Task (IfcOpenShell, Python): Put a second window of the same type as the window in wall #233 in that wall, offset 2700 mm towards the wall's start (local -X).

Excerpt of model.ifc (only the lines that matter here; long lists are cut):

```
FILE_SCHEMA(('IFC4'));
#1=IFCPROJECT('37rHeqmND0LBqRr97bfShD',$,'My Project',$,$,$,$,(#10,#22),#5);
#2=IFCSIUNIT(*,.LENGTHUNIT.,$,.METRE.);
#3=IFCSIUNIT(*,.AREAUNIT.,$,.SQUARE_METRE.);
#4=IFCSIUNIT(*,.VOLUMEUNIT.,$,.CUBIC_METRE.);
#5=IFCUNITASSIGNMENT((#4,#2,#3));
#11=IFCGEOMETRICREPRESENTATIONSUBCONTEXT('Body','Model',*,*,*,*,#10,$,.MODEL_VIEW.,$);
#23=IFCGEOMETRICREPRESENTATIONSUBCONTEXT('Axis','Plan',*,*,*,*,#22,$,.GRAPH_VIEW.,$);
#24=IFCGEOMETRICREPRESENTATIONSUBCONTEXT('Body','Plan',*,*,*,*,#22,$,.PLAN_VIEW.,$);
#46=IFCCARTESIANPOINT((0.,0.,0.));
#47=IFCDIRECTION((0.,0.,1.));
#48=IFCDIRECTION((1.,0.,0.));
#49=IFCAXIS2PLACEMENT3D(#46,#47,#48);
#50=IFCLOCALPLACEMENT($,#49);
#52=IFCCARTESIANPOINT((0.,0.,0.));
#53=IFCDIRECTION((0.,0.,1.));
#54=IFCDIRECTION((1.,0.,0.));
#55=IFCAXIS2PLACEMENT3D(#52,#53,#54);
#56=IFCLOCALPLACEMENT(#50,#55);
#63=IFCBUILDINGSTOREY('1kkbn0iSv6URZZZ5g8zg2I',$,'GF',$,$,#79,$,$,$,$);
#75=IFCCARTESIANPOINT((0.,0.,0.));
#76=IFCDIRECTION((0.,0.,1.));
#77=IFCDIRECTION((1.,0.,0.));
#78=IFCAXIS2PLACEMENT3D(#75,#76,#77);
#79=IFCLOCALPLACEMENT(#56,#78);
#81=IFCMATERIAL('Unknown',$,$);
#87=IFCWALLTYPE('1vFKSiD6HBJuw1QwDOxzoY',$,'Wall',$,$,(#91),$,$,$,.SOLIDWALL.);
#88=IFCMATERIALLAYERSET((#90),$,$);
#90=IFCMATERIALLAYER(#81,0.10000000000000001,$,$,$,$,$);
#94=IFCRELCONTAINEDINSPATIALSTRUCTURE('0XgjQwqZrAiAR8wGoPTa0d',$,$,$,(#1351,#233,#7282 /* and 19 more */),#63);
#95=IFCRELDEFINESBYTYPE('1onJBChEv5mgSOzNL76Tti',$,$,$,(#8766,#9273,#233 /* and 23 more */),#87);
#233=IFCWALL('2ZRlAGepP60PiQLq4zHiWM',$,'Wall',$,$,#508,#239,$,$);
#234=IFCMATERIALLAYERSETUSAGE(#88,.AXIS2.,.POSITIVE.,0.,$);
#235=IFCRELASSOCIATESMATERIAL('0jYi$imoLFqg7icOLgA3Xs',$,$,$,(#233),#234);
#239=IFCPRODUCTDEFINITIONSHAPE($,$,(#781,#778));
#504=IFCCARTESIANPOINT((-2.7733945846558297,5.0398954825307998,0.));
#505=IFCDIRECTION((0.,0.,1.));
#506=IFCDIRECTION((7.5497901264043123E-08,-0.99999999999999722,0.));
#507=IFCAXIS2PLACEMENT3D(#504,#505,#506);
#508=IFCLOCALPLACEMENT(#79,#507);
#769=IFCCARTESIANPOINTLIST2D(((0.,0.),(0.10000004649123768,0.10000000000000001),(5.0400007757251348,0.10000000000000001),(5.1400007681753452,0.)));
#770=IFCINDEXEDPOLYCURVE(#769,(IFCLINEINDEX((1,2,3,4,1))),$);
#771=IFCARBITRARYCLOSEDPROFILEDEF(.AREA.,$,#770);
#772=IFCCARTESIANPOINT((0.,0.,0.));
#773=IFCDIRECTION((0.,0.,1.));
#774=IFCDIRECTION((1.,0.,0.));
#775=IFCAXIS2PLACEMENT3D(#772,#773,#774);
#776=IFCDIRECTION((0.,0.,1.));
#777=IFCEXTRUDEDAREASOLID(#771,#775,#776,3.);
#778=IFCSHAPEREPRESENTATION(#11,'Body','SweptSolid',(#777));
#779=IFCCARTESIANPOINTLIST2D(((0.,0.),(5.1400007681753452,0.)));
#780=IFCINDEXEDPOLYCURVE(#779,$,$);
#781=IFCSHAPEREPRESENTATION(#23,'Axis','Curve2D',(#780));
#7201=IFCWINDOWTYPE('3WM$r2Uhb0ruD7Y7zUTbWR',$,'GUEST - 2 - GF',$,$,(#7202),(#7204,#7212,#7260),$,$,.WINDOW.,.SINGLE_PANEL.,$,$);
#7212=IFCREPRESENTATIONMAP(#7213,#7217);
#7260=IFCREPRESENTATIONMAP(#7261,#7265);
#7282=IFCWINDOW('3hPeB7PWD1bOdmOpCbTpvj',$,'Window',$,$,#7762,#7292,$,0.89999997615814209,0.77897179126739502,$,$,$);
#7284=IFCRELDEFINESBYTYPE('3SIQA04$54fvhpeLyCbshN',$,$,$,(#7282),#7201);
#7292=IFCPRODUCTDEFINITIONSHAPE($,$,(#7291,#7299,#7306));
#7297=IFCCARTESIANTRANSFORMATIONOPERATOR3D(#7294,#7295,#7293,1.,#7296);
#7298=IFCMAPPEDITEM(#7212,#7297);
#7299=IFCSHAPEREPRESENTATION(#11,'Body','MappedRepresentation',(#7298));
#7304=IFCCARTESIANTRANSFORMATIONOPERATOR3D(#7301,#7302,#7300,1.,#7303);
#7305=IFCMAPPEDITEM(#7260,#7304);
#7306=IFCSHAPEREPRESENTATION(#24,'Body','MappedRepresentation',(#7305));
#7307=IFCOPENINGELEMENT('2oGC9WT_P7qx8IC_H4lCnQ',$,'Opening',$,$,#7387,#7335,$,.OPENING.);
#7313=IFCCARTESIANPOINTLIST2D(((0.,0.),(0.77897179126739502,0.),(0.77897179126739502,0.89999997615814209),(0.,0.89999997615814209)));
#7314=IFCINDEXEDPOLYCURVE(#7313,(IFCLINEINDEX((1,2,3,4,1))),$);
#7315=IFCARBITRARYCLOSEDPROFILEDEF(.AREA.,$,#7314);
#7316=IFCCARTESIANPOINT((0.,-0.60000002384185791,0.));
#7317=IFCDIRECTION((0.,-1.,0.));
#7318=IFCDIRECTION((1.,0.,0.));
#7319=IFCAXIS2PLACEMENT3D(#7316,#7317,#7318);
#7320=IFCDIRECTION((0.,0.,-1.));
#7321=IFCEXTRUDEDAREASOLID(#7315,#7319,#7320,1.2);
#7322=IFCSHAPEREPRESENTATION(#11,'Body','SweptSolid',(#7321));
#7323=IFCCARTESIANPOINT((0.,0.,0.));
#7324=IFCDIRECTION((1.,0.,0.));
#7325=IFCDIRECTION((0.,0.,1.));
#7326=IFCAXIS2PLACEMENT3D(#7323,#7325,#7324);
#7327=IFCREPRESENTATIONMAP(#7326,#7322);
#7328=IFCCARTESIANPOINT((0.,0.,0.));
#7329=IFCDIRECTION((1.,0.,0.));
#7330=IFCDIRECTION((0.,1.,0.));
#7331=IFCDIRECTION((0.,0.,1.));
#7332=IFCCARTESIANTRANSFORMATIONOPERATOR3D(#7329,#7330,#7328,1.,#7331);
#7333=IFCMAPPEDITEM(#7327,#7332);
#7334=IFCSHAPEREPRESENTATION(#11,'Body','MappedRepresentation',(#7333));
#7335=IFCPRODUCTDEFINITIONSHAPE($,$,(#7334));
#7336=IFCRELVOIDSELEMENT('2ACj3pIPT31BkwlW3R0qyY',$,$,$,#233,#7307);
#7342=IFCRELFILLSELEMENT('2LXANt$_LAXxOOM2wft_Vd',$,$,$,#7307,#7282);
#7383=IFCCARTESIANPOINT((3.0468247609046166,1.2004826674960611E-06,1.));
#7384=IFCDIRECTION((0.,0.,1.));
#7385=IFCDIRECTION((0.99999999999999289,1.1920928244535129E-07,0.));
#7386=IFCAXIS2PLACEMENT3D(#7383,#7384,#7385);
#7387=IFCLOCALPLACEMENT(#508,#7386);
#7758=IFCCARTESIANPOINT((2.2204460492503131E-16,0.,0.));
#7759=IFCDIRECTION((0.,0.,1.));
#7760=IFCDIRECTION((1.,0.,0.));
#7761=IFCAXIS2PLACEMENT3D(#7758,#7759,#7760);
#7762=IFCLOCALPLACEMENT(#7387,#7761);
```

```python
import ifcopenshell
import ifcopenshell.api.feature
import ifcopenshell.api.geometry
import ifcopenshell.api.root
import ifcopenshell.geom
import ifcopenshell.util.element
import ifcopenshell.util.placement
import ifcopenshell.util.shape
import ifcopenshell.util.unit

model = ifcopenshell.open("model.ifc")
unit_scale = ifcopenshell.util.unit.calculate_unit_scale(model)
settings = ifcopenshell.geom.settings()


def volume(element):
    """Net volume in cubic metres, openings subtracted."""
    shape = ifcopenshell.geom.create_shape(settings, element)
    return ifcopenshell.util.shape.get_volume(shape.geometry)


window = model.by_guid("3hPeB7PWD1bOdmOpCbTpvj")
opening = window.FillsVoids[0].RelatingOpeningElement
wall = opening.VoidsElements[0].RelatingBuildingElement
before = volume(wall)
shift = ifcopenshell.util.placement.get_local_placement(wall.ObjectPlacement)[:3, 0] * -2.7 / unit_scale

# copy_class copies the void relationship, type, container and properties, but no geometry.
new_opening = ifcopenshell.api.root.copy_class(model, product=opening)
new_opening.Representation = ifcopenshell.util.element.copy_deep(
    model, opening.Representation, exclude=["IfcGeometricRepresentationContext", "IfcRepresentationMap"]
)
new_window = ifcopenshell.api.root.copy_class(model, product=window)
new_window.Representation = ifcopenshell.util.element.copy_deep(
    model, window.Representation, exclude=["IfcGeometricRepresentationContext", "IfcRepresentationMap"]
)
ifcopenshell.api.feature.add_filling(model, opening=new_opening, element=new_window)

for old, new in ((opening, new_opening), (window, new_window)):
    matrix = ifcopenshell.util.placement.get_local_placement(old.ObjectPlacement)
    matrix[:3, 3] += shift
    ifcopenshell.api.geometry.edit_object_placement(model, product=new, matrix=matrix, is_si=False)

after = volume(wall)

print(f"wall volume {before:.3f} -> {after:.3f} m3")

model.write("model-out.ifc")
```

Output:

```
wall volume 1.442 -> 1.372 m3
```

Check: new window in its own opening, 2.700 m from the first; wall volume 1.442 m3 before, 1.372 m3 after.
